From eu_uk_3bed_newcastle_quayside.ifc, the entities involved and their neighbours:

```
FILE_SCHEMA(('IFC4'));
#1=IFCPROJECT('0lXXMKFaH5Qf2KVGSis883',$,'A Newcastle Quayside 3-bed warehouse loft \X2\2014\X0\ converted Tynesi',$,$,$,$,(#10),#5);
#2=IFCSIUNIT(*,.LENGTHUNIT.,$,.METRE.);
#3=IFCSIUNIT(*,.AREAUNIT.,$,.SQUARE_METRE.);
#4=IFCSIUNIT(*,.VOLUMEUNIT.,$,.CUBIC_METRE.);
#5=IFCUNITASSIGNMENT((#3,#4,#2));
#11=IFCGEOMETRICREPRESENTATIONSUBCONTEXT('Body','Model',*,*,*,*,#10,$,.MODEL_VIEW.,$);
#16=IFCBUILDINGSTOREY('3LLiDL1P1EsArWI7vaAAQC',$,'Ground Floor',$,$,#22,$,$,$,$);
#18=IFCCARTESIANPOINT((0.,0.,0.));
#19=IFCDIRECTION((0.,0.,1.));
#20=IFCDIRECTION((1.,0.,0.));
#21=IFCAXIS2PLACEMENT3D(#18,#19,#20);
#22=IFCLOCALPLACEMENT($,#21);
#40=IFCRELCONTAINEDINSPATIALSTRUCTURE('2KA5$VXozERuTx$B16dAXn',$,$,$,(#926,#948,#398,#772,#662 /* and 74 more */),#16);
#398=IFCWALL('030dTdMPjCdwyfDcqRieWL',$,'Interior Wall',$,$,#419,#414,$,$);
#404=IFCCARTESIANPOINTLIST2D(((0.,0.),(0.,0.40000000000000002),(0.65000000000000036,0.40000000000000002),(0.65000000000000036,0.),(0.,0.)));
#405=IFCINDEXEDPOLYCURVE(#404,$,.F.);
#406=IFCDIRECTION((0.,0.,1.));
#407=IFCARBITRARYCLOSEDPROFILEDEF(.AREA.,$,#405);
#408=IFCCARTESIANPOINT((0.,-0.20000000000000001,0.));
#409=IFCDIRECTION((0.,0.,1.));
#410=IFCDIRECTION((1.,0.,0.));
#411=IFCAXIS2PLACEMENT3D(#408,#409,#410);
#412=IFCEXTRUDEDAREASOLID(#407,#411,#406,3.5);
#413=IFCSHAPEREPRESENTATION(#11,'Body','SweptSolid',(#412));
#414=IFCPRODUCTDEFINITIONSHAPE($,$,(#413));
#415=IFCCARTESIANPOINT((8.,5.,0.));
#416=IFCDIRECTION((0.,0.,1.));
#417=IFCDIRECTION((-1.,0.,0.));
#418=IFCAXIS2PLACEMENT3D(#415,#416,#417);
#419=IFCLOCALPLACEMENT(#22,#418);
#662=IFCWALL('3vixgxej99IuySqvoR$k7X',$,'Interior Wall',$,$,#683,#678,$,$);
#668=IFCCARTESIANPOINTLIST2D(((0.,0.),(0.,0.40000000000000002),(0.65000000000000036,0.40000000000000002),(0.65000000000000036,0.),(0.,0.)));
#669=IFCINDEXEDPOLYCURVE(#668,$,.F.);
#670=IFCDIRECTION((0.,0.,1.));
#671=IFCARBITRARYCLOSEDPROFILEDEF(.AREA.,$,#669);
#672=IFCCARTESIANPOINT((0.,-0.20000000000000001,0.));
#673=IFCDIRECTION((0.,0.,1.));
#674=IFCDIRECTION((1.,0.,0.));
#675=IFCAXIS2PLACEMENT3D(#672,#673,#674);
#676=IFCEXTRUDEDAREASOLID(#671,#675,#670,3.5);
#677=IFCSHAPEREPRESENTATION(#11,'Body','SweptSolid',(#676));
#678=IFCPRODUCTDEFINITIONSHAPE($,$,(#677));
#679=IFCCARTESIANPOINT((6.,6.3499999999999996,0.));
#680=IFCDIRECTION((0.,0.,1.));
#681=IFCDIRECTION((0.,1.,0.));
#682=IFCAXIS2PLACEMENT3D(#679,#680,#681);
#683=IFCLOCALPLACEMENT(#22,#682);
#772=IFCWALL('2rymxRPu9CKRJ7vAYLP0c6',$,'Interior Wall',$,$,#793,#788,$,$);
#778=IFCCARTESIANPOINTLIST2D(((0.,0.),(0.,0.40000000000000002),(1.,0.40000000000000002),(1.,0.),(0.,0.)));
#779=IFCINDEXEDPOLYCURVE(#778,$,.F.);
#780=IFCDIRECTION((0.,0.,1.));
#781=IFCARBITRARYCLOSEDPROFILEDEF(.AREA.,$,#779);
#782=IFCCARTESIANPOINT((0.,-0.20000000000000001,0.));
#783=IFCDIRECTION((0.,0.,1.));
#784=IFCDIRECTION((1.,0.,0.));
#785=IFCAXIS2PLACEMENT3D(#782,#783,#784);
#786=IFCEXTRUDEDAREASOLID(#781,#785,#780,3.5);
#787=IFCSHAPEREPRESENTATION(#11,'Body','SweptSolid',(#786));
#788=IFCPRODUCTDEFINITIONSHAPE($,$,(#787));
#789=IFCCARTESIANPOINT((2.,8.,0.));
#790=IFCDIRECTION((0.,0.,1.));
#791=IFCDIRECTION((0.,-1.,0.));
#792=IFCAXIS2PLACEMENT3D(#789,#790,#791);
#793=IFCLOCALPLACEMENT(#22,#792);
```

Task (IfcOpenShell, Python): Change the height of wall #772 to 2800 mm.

```python
import ifcopenshell
import ifcopenshell.geom
import ifcopenshell.util.representation
import ifcopenshell.util.shape

model = ifcopenshell.open("eu_uk_3bed_newcastle_quayside.ifc")
settings = ifcopenshell.geom.settings()


def volume(element):
    """Net volume in cubic metres, openings subtracted."""
    shape = ifcopenshell.geom.create_shape(settings, element)
    return ifcopenshell.util.shape.get_volume(shape.geometry)


wall = model.by_guid("2rymxRPu9CKRJ7vAYLP0c6")
before = volume(wall)

body = ifcopenshell.util.representation.get_representation(wall, "Model", "Body")
solid = body.Items[0]
old_height = solid.Depth
solid.Depth = 2.8
after = volume(wall)

print(f"height {old_height:g} -> {solid.Depth:g}, volume {before:.3f} -> {after:.3f} m3")

model.write("eu_uk_3bed_newcastle_quayside-out.ifc")
```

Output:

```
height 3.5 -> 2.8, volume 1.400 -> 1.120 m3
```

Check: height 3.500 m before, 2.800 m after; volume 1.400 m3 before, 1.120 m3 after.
